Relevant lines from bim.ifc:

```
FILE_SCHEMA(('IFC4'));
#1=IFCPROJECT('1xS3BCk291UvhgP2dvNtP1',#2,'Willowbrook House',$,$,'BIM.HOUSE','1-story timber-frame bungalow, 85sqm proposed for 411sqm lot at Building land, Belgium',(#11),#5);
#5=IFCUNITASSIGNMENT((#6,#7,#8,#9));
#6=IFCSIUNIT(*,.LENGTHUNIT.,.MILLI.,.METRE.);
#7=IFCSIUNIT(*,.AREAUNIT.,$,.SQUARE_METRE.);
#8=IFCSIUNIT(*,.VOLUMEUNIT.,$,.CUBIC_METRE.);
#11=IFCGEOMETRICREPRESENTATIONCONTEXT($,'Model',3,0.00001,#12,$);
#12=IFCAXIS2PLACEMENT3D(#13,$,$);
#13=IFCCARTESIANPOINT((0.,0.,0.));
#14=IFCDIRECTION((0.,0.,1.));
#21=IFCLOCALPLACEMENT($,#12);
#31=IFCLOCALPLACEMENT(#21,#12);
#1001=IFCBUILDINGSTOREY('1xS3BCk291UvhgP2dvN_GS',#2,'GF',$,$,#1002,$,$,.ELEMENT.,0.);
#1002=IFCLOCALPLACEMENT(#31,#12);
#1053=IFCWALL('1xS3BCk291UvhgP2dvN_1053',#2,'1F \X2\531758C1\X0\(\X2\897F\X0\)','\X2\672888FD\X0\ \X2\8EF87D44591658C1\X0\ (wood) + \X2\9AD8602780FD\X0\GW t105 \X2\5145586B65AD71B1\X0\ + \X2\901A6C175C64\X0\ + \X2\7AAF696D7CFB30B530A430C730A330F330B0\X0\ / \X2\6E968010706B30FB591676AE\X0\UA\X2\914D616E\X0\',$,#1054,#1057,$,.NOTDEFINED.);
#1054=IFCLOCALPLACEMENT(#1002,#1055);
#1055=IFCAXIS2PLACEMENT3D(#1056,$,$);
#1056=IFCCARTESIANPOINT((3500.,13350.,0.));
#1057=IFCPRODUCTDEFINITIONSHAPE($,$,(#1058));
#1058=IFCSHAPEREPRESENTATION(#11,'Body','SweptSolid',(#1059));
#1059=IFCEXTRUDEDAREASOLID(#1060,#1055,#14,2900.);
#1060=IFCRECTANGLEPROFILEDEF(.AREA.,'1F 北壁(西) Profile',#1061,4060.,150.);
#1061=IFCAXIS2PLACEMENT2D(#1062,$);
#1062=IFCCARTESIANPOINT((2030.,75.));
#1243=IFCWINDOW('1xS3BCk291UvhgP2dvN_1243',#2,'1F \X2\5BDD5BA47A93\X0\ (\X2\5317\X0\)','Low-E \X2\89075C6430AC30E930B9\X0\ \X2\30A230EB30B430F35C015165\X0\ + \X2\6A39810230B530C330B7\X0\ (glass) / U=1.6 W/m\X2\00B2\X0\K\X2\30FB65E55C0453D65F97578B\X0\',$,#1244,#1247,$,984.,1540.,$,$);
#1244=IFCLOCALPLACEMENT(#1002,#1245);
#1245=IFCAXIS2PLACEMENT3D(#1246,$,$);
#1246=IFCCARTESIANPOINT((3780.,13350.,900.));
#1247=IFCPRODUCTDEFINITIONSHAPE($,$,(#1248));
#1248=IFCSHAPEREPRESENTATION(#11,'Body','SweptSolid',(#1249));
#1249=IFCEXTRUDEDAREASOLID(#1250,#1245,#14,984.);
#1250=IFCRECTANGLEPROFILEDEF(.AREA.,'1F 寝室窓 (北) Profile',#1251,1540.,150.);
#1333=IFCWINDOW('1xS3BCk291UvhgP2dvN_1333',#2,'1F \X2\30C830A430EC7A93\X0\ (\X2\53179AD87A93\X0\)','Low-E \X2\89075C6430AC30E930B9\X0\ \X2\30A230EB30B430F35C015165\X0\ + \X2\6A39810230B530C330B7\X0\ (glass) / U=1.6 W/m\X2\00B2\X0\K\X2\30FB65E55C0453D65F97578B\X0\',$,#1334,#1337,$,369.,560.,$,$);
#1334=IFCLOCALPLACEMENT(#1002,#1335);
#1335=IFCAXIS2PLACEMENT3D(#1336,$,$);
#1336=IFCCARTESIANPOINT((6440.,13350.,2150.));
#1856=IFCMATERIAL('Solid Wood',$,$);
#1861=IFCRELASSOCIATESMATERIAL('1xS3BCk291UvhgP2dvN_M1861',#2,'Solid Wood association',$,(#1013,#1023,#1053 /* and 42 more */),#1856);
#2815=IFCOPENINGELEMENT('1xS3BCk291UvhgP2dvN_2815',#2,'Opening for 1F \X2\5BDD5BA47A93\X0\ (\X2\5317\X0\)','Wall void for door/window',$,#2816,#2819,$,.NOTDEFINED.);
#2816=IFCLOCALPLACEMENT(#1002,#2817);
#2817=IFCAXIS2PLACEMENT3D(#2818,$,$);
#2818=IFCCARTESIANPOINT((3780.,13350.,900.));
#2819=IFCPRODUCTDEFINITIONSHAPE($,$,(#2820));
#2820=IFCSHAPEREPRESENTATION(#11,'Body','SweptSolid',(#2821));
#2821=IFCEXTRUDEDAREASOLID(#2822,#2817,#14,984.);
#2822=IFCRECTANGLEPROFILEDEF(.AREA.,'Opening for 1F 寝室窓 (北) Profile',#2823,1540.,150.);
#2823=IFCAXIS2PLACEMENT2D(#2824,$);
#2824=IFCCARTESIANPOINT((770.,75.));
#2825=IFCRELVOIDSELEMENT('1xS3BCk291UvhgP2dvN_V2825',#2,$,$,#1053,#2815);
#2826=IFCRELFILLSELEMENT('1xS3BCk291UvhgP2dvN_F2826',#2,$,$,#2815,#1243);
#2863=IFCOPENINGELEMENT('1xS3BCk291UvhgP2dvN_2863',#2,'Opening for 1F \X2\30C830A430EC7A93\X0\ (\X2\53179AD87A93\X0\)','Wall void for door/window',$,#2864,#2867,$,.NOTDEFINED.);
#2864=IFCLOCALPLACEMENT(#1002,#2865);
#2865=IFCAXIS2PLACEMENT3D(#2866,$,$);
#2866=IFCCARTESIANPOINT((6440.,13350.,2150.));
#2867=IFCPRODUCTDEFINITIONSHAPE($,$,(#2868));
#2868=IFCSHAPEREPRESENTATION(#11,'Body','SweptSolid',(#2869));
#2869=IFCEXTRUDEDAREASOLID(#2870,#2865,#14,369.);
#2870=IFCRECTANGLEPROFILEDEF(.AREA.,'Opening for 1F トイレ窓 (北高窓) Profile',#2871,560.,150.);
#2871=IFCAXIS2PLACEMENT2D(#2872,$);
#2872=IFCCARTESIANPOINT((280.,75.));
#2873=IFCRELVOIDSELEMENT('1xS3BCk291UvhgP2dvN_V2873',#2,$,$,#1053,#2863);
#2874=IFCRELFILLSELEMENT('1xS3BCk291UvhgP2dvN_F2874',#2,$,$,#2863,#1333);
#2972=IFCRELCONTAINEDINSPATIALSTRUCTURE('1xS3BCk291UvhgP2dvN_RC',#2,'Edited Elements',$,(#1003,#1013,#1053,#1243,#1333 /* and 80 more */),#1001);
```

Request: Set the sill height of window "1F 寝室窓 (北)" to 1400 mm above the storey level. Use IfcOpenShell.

```python
import numpy as np
import ifcopenshell
import ifcopenshell.api.geometry
import ifcopenshell.geom
import ifcopenshell.util.element
import ifcopenshell.util.placement
import ifcopenshell.util.shape
import ifcopenshell.util.unit

model = ifcopenshell.open("bim.ifc")
unit_scale = ifcopenshell.util.unit.calculate_unit_scale(model)

window = model.by_id(1243)
opening = window.FillsVoids[0].RelatingOpeningElement
storey = ifcopenshell.util.element.get_container(window, ifc_class="IfcBuildingStorey")
level = ifcopenshell.util.placement.get_local_placement(storey.ObjectPlacement)[2, 3]

# The opening's origin need not be at the sill, so measure its lowest point.
shape = ifcopenshell.geom.create_shape(ifcopenshell.geom.settings(), opening)
bottom = ifcopenshell.util.shape.get_shape_bottom_elevation(shape, shape.geometry) / unit_scale
dz = level + 1400.0 - bottom

shift = np.array([0.0, 0.0, dz])
# The window is not placed relative to its opening, so move both.
for product in (opening, window):
    matrix = ifcopenshell.util.placement.get_local_placement(product.ObjectPlacement)
    matrix[:3, 3] += shift
    ifcopenshell.api.geometry.edit_object_placement(model, product=product, matrix=matrix, is_si=False)

print(f"moved by {dz * unit_scale:+.3f} m")

model.write("bim_updated.ifc")
```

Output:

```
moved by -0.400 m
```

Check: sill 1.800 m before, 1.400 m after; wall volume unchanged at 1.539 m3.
